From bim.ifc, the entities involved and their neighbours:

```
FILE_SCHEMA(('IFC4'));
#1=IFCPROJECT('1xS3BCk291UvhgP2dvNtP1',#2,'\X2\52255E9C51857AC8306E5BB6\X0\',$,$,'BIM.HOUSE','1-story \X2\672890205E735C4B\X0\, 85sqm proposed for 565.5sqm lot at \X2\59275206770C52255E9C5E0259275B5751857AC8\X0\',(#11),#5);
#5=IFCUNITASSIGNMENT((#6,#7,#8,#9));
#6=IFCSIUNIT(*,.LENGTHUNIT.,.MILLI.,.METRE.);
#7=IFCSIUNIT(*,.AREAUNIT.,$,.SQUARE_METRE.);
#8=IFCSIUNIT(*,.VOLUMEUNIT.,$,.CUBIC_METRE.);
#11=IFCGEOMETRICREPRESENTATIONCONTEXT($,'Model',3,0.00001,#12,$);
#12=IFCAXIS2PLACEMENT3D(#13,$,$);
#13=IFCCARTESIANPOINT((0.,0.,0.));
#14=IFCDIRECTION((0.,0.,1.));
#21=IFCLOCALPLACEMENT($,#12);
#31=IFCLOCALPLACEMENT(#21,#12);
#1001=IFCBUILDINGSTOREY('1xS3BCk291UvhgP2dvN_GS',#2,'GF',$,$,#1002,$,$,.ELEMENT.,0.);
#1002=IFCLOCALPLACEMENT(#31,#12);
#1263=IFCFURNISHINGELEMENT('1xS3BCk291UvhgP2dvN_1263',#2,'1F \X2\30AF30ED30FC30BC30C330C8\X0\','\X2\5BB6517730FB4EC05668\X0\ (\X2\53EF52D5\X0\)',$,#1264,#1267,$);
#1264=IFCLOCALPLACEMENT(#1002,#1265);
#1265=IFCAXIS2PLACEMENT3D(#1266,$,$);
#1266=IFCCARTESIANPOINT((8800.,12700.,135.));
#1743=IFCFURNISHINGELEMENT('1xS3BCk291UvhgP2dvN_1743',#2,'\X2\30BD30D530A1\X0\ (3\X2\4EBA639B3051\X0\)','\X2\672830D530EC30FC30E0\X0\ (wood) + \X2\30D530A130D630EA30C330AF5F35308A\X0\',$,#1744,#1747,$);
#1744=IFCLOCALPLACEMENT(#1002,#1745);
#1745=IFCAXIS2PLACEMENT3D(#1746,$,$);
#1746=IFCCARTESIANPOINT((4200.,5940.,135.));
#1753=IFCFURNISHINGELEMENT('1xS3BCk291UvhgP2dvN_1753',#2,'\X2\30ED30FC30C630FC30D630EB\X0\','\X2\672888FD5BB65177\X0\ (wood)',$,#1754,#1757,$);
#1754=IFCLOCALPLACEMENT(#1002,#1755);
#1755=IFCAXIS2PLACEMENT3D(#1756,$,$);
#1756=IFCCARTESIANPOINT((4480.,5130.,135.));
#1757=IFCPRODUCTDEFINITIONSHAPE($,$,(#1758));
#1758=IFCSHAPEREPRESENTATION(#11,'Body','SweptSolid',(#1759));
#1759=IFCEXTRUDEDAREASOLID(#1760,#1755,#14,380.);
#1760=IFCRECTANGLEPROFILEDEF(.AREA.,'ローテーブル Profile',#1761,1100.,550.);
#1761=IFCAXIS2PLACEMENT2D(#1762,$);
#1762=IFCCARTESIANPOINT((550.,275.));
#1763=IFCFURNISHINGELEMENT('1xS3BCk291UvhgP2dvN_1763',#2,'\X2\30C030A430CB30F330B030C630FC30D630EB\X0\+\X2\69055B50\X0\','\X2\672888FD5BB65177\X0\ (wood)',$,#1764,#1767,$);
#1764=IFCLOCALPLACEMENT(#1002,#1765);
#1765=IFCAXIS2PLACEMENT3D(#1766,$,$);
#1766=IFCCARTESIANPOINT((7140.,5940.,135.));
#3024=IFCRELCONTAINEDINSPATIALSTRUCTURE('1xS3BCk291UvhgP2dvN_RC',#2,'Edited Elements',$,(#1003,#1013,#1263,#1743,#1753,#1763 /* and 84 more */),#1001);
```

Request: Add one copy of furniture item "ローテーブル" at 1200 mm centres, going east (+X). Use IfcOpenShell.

```python
import numpy as np
import ifcopenshell
import ifcopenshell.api.geometry
import ifcopenshell.api.root
import ifcopenshell.util.element
import ifcopenshell.util.placement
import ifcopenshell.util.unit

model = ifcopenshell.open("bim.ifc")
unit_scale = ifcopenshell.util.unit.calculate_unit_scale(model)


def reuse_history(source, copy):
    """copy_class also copies each property set's owner history, people and application; keep the originals."""
    for rel in copy.IsDefinedBy:
        if rel.is_a("IfcRelDefinesByProperties") and (history := rel.RelatingPropertyDefinition.OwnerHistory):
            rel.RelatingPropertyDefinition.OwnerHistory = source.OwnerHistory
            ifcopenshell.util.element.remove_deep2(model, history)


source = model.by_id(1753)
base = ifcopenshell.util.placement.get_local_placement(source.ObjectPlacement)
step = np.array([1.0, 0.0, 0.0]) * 1.2 / unit_scale

for i in range(1, 2):
    copy = ifcopenshell.api.root.copy_class(model, product=source)
    copy.Representation = ifcopenshell.util.element.copy_deep(
        model, source.Representation, exclude=["IfcGeometricRepresentationContext", "IfcRepresentationMap"]
    )
    reuse_history(source, copy)
    matrix = base.copy()
    matrix[:3, 3] += i * step
    print("added at", matrix[:3, 3].round(3) + 0.0)
    ifcopenshell.api.geometry.edit_object_placement(model, product=copy, matrix=matrix, is_si=False)

model.write("bim_v2.ifc")
```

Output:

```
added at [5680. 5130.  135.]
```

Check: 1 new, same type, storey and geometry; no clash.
